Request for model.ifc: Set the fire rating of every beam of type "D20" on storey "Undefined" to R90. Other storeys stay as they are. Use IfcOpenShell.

First a look at what the model holds.

```python
import ifcopenshell
import ifcopenshell.util.element

model = ifcopenshell.open("model.ifc")
print(model.schema)
storey = next(s for s in model.by_type("IfcBuildingStorey") if s.Name == "Undefined")
beams = [e for e in ifcopenshell.util.element.get_decomposition(storey) if e.is_a("IfcBeam")]
seen = {}
for e in beams:
    element_type = ifcopenshell.util.element.get_type(e)
    key = (element_type.Name if element_type != e and element_type else None, ifcopenshell.util.element.get_pset(e, "Pset_BeamCommon", "FireRating"))
    seen[key] = seen.get(key, 0) + 1
for (name, value), count in sorted(seen.items(), key=str):
    print(count, "x", name, "|", value)
```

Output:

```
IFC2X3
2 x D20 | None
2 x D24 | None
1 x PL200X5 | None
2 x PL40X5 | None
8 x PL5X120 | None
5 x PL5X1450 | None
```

```python
import ifcopenshell
import ifcopenshell.api.pset
import ifcopenshell.util.element

model = ifcopenshell.open("model.ifc")

storey = next(s for s in model.by_type("IfcBuildingStorey") if s.Name == "Undefined")
beams = [e for e in ifcopenshell.util.element.get_decomposition(storey) if e.is_a("IfcBeam")]

count = 0
for e in beams:
    element_type = ifcopenshell.util.element.get_type(e)
    if element_type in (None, e) or element_type.Name != "D20":
        continue
    # add_pset returns the element's existing set when there is one.
    pset = ifcopenshell.api.pset.add_pset(model, product=e, name="Pset_BeamCommon")
    ifcopenshell.api.pset.edit_pset(model, pset=pset, properties={"FireRating": "R90"})
    count += 1

print(count, "beams updated")

model.write("model_edited.ifc")
```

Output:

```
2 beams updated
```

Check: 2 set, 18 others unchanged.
